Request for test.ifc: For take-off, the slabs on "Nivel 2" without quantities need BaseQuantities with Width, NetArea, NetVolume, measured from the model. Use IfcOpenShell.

First a look at what the model holds.

```python
import ifcopenshell
import ifcopenshell.util.element
import ifcopenshell.util.unit

model = ifcopenshell.open("test.ifc")
print(model.schema)
for unit_type in ("LENGTHUNIT", "AREAUNIT", "VOLUMEUNIT"):
    print(unit_type, ifcopenshell.util.unit.calculate_unit_scale(model, unit_type))
storey = next(s for s in model.by_type("IfcBuildingStorey") if s.Name == "Nivel 2")
slabs = [e for e in ifcopenshell.util.element.get_decomposition(storey) if e.is_a("IfcSlab")]
for e in sorted(slabs, key=lambda e: e.id()):
    print(e.id(), e.is_a(), e.Name, list(ifcopenshell.util.element.get_psets(e, qtos_only=True)), sep=" | ")
```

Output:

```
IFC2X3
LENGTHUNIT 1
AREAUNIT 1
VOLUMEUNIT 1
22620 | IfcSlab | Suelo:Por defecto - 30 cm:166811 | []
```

```python
import ifcopenshell
import ifcopenshell.api.pset
import ifcopenshell.geom
import ifcopenshell.util.element
import ifcopenshell.util.shape
import ifcopenshell.util.unit

model = ifcopenshell.open("test.ifc")
unit_scale = ifcopenshell.util.unit.calculate_unit_scale(model)
area_scale = ifcopenshell.util.unit.calculate_unit_scale(model, "AREAUNIT")
volume_scale = ifcopenshell.util.unit.calculate_unit_scale(model, "VOLUMEUNIT")
settings = ifcopenshell.geom.settings()

storey = next(s for s in model.by_type("IfcBuildingStorey") if s.Name == "Nivel 2")
slabs = [e for e in ifcopenshell.util.element.get_decomposition(storey) if e.is_a("IfcSlab")]

for e in sorted(slabs, key=lambda e: e.id()):
    if ifcopenshell.util.element.get_psets(e, qtos_only=True, should_inherit=False):
        continue
    # Geometry comes back in metres, in the element's own axes.
    shape = ifcopenshell.geom.create_shape(settings, e)
    values = {
        "Width": ifcopenshell.util.shape.get_z(shape.geometry) / unit_scale,
        "NetArea": ifcopenshell.util.shape.get_footprint_area(shape.geometry) / area_scale,
        "NetVolume": ifcopenshell.util.shape.get_volume(shape.geometry) / volume_scale,
    }
    qto = ifcopenshell.api.pset.add_qto(model, product=e, name="BaseQuantities")
    ifcopenshell.api.pset.edit_qto(model, qto=qto, properties=values)
    print(e.id(), {k: round(v, 3) for k, v in values.items()})

model.write("test_v2.ifc")
```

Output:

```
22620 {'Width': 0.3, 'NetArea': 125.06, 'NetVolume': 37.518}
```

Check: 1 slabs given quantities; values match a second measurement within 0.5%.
